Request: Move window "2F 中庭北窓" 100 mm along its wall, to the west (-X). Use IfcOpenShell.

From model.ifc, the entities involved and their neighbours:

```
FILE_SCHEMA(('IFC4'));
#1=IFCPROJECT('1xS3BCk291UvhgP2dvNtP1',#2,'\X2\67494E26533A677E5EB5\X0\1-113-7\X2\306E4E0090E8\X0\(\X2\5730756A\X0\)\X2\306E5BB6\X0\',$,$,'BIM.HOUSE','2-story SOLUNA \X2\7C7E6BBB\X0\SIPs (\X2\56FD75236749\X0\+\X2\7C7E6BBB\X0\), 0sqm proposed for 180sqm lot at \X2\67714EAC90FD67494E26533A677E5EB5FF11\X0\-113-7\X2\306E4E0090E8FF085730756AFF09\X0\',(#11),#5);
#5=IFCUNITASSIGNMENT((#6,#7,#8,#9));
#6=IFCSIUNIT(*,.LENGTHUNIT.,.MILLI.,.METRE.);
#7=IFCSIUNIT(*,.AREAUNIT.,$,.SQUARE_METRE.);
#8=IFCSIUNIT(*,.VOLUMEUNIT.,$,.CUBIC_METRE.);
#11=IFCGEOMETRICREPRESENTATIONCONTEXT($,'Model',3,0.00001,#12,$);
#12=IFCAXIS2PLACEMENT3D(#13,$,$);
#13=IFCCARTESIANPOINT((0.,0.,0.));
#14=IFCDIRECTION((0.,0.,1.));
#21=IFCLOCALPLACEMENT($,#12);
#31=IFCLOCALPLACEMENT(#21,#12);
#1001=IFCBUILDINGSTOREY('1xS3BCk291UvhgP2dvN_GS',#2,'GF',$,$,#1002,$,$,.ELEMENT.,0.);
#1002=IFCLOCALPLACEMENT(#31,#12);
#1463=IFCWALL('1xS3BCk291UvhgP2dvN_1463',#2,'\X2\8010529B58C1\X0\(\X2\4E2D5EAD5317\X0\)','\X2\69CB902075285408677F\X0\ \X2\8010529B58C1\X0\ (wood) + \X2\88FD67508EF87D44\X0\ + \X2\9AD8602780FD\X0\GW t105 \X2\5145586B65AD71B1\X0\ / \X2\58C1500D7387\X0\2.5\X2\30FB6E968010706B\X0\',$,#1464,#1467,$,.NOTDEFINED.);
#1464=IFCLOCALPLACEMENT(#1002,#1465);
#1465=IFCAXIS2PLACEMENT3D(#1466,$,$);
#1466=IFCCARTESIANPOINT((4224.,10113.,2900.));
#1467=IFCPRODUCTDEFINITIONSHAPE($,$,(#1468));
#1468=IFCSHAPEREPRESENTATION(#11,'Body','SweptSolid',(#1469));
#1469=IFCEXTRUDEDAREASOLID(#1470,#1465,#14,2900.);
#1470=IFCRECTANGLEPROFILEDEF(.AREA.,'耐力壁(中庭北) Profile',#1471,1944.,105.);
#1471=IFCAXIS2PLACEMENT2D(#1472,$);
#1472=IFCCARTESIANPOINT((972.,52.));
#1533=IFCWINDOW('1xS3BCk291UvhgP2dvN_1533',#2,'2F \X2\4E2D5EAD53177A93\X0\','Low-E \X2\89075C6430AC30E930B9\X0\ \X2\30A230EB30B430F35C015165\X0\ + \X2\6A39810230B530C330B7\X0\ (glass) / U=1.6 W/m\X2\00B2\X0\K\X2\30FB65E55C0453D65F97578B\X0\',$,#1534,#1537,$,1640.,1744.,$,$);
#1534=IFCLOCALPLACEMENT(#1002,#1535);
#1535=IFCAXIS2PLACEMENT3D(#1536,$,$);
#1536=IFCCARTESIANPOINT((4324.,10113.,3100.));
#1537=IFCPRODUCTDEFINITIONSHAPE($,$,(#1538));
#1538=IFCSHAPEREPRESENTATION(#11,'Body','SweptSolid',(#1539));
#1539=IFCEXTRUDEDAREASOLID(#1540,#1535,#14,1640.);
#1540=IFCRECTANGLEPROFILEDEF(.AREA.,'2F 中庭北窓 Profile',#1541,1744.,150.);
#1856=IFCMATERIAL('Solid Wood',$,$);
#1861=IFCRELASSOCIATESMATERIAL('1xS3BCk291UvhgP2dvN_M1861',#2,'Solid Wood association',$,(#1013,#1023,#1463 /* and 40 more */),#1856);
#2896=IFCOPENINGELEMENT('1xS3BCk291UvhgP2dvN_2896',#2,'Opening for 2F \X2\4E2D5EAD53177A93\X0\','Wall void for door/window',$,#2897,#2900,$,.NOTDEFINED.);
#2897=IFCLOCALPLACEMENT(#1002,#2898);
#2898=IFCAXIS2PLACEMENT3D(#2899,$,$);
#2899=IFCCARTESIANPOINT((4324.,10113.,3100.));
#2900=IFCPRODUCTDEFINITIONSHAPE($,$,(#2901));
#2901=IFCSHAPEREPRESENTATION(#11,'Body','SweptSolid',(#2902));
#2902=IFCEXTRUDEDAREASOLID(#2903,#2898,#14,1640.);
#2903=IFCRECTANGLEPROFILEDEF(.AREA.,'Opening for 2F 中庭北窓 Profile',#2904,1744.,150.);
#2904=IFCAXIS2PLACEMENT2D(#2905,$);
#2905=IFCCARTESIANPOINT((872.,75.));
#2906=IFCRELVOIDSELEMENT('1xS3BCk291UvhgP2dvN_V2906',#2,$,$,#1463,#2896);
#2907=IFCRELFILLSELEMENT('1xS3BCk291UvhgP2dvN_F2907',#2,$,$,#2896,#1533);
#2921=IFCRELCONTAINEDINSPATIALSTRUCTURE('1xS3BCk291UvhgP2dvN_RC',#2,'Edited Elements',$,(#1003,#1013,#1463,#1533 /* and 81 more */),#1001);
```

```python
import ifcopenshell
import ifcopenshell.api.geometry
import ifcopenshell.util.placement
import ifcopenshell.util.unit

model = ifcopenshell.open("model.ifc")
unit_scale = ifcopenshell.util.unit.calculate_unit_scale(model)

window = model.by_guid("1xS3BCk291UvhgP2dvN_1533")
opening = window.FillsVoids[0].RelatingOpeningElement
wall = opening.VoidsElements[0].RelatingBuildingElement

wall_matrix = ifcopenshell.util.placement.get_local_placement(wall.ObjectPlacement)
shift = wall_matrix[:3, 0] * -0.1 / unit_scale
before = ifcopenshell.util.placement.get_local_placement(window.ObjectPlacement)[:3, 3].copy()

# The window is not placed relative to its opening, so move both.
for product in (opening, window):
    matrix = ifcopenshell.util.placement.get_local_placement(product.ObjectPlacement)
    matrix[:3, 3] += shift
    ifcopenshell.api.geometry.edit_object_placement(model, product=product, matrix=matrix, is_si=False)

after = ifcopenshell.util.placement.get_local_placement(window.ObjectPlacement)[:3, 3]
print("window moved by", (after - before).round(3) + 0.0)

model.write("model_updated.ifc")
```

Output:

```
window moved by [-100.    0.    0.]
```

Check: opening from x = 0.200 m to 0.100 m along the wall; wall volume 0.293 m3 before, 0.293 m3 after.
